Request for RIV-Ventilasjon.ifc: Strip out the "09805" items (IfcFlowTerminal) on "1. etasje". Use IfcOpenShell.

First a look at what the model holds.

```python
import ifcopenshell
import ifcopenshell.util.element

model = ifcopenshell.open("RIV-Ventilasjon.ifc")
print(model.schema)
storey = next(s for s in model.by_type("IfcBuildingStorey") if s.Name == "1. etasje")
terminals = [e for e in ifcopenshell.util.element.get_decomposition(storey) if e.is_a("IfcFlowTerminal")]
seen = {}
for e in terminals:
    element_type = ifcopenshell.util.element.get_type(e)
    name = element_type.Name if element_type not in (None, e) else None
    seen[name] = seen.get(name, 0) + 1
for name, count in sorted(seen.items(), key=str):
    print(count, "x", name)
```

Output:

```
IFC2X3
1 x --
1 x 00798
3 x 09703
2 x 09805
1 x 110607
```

```python
import ifcopenshell
import ifcopenshell.api.root
import ifcopenshell.util.element

model = ifcopenshell.open("RIV-Ventilasjon.ifc")

storey = next(s for s in model.by_type("IfcBuildingStorey") if s.Name == "1. etasje")
terminals = [e for e in ifcopenshell.util.element.get_decomposition(storey) if e.is_a("IfcFlowTerminal")]
targets = [e for e in terminals if (t := ifcopenshell.util.element.get_type(e)) not in (None, e) and t.Name == "09805"]

for e in targets:
    ifcopenshell.api.root.remove_product(model, product=e)
print(len(targets), "removed")

model.write("RIV-Ventilasjon_edited.ifc")
```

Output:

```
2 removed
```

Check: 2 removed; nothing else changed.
